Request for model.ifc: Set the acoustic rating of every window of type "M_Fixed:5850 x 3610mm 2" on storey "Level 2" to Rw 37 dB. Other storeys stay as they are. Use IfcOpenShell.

First a look at what the model holds.

```python
import ifcopenshell
import ifcopenshell.util.element

model = ifcopenshell.open("model.ifc")
print(model.schema)
storey = next(s for s in model.by_type("IfcBuildingStorey") if s.Name == "Level 2")
windows = [e for e in ifcopenshell.util.element.get_decomposition(storey) if e.is_a("IfcWindow")]
seen = {}
for e in windows:
    element_type = ifcopenshell.util.element.get_type(e)
    key = (element_type.Name if element_type != e and element_type else None, ifcopenshell.util.element.get_pset(e, "Pset_WindowCommon", "AcousticRating"))
    seen[key] = seen.get(key, 0) + 1
for (name, value), count in sorted(seen.items(), key=str):
    print(count, "x", name, "|", value)
```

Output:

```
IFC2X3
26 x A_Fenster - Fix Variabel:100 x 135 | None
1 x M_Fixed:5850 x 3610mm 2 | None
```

```python
import ifcopenshell
import ifcopenshell.api.pset
import ifcopenshell.util.element

model = ifcopenshell.open("model.ifc")

storey = next(s for s in model.by_type("IfcBuildingStorey") if s.Name == "Level 2")
windows = [e for e in ifcopenshell.util.element.get_decomposition(storey) if e.is_a("IfcWindow")]

count = 0
for e in windows:
    element_type = ifcopenshell.util.element.get_type(e)
    if element_type in (None, e) or element_type.Name != "M_Fixed:5850 x 3610mm 2":
        continue
    # add_pset returns the element's existing set when there is one.
    pset = ifcopenshell.api.pset.add_pset(model, product=e, name="Pset_WindowCommon")
    ifcopenshell.api.pset.edit_pset(model, pset=pset, properties={"AcousticRating": "Rw 37 dB"})
    count += 1

print(count, "windows updated")

model.write("model_v2.ifc")
```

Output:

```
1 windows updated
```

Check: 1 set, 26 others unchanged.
